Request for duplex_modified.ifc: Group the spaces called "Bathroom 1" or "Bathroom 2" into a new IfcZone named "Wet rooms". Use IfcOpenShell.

First a look at what the model holds.

```python
import ifcopenshell

model = ifcopenshell.open("duplex_modified.ifc")
print(model.schema)
seen = {}
for space in model.by_type("IfcSpace"):
    seen[space.LongName] = seen.get(space.LongName, 0) + 1
for name, count in sorted(seen.items(), key=str):
    print(count, "x", name)
print("zones:", [z.Name for z in model.by_type("IfcZone")][:20])
```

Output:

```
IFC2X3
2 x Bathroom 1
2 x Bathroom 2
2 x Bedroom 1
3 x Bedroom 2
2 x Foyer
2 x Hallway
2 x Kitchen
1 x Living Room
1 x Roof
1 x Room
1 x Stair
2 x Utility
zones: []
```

```python
import ifcopenshell
import ifcopenshell.api.group
import ifcopenshell.api.root

model = ifcopenshell.open("duplex_modified.ifc")

names = {"Bathroom 1", "Bathroom 2"}
spaces = [s for s in model.by_type("IfcSpace") if s.LongName in names]

zone = ifcopenshell.api.root.create_entity(model, ifc_class="IfcZone", name="Wet rooms")
ifcopenshell.api.group.assign_group(model, products=spaces, group=zone)
print(len(spaces), "spaces in", zone.Name)

model.write("duplex_modified_updated.ifc")
```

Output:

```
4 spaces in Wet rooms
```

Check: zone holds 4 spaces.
